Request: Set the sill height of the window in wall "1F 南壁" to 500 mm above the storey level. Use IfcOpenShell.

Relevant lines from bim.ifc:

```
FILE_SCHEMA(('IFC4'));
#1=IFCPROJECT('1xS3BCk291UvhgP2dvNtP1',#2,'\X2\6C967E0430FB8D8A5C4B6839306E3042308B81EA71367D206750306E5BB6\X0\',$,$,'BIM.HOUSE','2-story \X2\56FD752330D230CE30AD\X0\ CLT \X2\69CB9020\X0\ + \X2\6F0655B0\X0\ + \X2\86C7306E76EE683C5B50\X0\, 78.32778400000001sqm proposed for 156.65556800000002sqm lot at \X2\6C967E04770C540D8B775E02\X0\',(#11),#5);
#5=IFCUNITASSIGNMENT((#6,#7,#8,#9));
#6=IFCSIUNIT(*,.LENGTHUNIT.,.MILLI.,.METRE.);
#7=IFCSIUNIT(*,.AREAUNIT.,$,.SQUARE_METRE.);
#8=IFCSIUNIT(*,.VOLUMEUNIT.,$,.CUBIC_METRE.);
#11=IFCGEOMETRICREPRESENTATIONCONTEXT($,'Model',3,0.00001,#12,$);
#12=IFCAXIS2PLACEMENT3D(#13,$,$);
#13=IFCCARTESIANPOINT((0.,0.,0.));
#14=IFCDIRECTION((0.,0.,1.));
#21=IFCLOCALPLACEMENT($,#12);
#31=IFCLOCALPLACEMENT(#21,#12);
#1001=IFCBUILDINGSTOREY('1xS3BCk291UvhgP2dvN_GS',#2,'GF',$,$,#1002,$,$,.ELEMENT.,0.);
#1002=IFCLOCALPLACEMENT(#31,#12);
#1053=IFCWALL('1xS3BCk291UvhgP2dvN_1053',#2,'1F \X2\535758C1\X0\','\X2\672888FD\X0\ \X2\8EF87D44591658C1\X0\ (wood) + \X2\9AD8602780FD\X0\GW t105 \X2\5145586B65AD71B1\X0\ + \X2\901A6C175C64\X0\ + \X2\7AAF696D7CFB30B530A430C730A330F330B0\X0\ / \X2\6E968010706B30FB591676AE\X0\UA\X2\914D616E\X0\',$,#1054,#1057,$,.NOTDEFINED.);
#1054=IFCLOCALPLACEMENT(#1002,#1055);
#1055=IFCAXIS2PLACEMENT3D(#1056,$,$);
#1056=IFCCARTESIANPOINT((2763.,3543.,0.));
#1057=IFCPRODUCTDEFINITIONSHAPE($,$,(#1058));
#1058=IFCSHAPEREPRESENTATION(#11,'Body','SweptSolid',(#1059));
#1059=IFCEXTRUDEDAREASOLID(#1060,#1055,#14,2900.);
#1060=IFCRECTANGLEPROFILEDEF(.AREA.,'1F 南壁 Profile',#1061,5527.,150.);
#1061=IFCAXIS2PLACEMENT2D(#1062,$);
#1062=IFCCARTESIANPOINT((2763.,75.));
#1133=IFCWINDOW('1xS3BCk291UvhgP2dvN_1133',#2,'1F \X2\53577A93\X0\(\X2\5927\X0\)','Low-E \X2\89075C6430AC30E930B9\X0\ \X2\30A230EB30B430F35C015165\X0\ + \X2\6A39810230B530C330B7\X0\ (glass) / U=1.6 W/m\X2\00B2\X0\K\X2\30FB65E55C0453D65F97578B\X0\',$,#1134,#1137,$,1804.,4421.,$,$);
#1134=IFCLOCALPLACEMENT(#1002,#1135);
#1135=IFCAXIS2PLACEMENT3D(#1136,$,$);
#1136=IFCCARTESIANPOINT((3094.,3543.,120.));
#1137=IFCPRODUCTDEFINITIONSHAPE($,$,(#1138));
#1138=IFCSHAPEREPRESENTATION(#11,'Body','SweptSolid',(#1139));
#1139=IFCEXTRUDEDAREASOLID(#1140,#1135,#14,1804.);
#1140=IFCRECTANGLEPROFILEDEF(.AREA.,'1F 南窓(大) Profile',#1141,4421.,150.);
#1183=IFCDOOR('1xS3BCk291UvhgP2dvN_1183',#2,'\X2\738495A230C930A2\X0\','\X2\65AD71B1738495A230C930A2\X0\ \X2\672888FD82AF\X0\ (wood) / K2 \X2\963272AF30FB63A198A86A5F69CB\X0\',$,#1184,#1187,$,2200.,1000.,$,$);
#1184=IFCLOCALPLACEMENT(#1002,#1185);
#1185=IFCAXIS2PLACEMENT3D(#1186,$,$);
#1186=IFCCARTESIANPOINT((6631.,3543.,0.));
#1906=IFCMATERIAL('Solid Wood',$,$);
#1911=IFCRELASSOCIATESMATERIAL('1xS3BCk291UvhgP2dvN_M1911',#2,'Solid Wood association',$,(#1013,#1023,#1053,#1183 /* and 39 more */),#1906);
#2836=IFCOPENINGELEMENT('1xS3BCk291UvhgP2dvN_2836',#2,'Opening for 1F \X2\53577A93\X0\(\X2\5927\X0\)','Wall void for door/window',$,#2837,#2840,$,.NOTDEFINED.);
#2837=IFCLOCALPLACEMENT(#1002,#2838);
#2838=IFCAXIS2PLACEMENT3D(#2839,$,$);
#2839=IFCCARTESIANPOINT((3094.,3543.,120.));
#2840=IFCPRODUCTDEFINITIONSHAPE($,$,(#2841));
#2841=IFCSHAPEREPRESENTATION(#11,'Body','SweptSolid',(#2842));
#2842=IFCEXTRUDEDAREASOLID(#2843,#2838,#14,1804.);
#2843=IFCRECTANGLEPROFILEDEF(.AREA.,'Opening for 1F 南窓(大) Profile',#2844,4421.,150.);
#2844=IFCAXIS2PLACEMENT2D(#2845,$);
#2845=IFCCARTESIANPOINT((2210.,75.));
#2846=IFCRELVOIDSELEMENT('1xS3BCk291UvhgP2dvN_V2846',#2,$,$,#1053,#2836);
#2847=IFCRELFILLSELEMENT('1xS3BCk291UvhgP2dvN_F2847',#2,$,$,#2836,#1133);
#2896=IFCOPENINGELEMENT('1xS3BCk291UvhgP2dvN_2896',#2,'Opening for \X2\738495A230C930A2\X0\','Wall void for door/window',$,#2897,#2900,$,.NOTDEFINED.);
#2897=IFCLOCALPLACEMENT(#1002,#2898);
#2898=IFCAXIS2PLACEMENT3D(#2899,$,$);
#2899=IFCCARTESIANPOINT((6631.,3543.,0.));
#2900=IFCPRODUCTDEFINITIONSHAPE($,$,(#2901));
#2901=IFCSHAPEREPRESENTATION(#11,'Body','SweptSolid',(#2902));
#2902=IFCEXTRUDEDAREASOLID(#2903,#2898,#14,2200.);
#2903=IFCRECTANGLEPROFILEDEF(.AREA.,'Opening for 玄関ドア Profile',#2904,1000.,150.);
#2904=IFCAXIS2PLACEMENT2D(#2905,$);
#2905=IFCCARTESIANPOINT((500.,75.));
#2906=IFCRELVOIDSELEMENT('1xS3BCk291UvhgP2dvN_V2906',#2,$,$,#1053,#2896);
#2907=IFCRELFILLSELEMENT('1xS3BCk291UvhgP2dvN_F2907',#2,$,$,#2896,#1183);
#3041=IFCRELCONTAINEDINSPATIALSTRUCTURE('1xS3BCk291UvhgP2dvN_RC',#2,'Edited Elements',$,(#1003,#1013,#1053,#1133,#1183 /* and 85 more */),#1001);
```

```python
import numpy as np
import ifcopenshell
import ifcopenshell.api.geometry
import ifcopenshell.geom
import ifcopenshell.util.element
import ifcopenshell.util.placement
import ifcopenshell.util.shape
import ifcopenshell.util.unit

model = ifcopenshell.open("bim.ifc")
unit_scale = ifcopenshell.util.unit.calculate_unit_scale(model)

window = model.by_id(1133)
opening = window.FillsVoids[0].RelatingOpeningElement
storey = ifcopenshell.util.element.get_container(window, ifc_class="IfcBuildingStorey")
level = ifcopenshell.util.placement.get_local_placement(storey.ObjectPlacement)[2, 3]

# The opening's origin need not be at the sill, so measure its lowest point.
shape = ifcopenshell.geom.create_shape(ifcopenshell.geom.settings(), opening)
bottom = ifcopenshell.util.shape.get_shape_bottom_elevation(shape, shape.geometry) / unit_scale
dz = level + 500.0 - bottom

shift = np.array([0.0, 0.0, dz])
# The window is not placed relative to its opening, so move both.
for product in (opening, window):
    matrix = ifcopenshell.util.placement.get_local_placement(product.ObjectPlacement)
    matrix[:3, 3] += shift
    ifcopenshell.api.geometry.edit_object_placement(model, product=product, matrix=matrix, is_si=False)

print(f"moved by {dz * unit_scale:+.3f} m")

model.write("bim_v2.ifc")
```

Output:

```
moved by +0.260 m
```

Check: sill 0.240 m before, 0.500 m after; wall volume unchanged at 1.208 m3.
